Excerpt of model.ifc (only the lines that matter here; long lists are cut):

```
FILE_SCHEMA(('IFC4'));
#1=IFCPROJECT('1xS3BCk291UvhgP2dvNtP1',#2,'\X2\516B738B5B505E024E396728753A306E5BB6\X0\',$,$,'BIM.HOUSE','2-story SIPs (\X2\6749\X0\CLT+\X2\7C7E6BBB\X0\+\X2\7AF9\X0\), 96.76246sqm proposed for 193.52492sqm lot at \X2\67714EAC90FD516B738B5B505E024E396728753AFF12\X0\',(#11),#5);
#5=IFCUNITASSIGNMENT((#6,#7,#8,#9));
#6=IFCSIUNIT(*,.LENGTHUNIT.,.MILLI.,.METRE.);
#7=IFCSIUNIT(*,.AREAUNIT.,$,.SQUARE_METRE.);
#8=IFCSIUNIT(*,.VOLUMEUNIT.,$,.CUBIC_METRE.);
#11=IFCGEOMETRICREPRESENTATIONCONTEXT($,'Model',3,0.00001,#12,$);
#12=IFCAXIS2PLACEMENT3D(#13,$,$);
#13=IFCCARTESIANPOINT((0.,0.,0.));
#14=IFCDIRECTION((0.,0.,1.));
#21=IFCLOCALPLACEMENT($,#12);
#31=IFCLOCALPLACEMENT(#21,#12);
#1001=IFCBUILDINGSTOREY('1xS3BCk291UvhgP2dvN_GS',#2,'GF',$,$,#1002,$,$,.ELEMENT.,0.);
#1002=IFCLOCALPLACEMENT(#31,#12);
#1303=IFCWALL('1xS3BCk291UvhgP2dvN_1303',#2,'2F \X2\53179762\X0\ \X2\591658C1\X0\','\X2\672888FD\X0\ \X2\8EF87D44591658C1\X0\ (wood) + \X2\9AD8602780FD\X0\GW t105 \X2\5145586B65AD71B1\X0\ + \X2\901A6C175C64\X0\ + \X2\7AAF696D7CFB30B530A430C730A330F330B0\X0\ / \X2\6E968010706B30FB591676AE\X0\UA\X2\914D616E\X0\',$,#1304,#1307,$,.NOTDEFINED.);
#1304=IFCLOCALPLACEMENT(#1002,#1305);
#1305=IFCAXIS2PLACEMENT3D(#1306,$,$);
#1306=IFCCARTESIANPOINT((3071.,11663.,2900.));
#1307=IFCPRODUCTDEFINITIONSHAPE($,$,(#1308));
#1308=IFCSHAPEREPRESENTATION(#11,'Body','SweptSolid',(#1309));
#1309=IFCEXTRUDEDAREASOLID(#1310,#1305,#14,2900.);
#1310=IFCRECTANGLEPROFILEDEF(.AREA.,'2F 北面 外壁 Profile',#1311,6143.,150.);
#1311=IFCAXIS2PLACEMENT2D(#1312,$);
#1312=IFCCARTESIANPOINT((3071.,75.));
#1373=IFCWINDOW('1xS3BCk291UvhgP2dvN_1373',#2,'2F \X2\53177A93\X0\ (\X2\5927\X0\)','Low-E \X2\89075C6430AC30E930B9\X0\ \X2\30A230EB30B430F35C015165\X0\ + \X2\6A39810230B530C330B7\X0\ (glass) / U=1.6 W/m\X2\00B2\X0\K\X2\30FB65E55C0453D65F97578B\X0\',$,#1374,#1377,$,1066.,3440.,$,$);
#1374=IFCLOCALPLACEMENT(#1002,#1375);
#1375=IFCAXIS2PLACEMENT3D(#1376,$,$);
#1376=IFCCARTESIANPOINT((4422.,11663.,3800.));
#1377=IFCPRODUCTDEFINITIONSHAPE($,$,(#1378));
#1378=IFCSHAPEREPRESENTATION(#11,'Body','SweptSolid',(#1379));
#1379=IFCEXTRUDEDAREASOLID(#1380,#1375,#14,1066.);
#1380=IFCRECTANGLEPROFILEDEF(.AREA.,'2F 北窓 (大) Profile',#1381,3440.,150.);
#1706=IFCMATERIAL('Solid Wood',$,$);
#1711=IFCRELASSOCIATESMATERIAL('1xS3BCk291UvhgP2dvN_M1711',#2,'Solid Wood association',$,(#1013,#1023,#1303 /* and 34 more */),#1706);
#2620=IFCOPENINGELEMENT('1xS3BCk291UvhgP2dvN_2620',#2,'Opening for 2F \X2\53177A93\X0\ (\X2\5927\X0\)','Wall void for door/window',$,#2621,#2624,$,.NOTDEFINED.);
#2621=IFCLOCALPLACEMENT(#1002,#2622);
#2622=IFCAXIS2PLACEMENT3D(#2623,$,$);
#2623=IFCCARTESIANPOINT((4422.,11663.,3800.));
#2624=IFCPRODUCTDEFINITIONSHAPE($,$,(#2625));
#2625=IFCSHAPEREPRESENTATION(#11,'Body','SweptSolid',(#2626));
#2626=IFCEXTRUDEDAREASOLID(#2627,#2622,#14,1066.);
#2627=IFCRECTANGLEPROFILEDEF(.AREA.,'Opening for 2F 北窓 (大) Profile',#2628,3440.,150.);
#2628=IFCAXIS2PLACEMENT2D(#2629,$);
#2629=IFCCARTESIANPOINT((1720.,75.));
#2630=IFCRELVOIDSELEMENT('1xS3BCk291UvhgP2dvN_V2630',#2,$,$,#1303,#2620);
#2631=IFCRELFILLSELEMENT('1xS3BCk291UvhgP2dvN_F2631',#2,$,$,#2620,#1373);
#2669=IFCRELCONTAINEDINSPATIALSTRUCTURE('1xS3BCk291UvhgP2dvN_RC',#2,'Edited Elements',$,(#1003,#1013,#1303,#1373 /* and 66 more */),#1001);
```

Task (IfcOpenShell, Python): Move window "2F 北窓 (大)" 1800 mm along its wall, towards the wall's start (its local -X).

```python
import ifcopenshell
import ifcopenshell.api.geometry
import ifcopenshell.util.placement

model = ifcopenshell.open("model.ifc")

window = model.by_id(1373)
opening = window.FillsVoids[0].RelatingOpeningElement
wall = opening.VoidsElements[0].RelatingBuildingElement

wall_matrix = ifcopenshell.util.placement.get_local_placement(wall.ObjectPlacement)
shift = wall_matrix[:3, 0] * -1800.0
before = ifcopenshell.util.placement.get_local_placement(window.ObjectPlacement)[:3, 3].copy()

# The window is not placed relative to its opening, so move both.
for product in (opening, window):
    matrix = ifcopenshell.util.placement.get_local_placement(product.ObjectPlacement)
    matrix[:3, 3] += shift
    ifcopenshell.api.geometry.edit_object_placement(model, product=product, matrix=matrix, is_si=False)

after = ifcopenshell.util.placement.get_local_placement(window.ObjectPlacement)[:3, 3]
print("window moved by", (after - before).round(3) + 0.0)

model.write("model_updated.ifc")
```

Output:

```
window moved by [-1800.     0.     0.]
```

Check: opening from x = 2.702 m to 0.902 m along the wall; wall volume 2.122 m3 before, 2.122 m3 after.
